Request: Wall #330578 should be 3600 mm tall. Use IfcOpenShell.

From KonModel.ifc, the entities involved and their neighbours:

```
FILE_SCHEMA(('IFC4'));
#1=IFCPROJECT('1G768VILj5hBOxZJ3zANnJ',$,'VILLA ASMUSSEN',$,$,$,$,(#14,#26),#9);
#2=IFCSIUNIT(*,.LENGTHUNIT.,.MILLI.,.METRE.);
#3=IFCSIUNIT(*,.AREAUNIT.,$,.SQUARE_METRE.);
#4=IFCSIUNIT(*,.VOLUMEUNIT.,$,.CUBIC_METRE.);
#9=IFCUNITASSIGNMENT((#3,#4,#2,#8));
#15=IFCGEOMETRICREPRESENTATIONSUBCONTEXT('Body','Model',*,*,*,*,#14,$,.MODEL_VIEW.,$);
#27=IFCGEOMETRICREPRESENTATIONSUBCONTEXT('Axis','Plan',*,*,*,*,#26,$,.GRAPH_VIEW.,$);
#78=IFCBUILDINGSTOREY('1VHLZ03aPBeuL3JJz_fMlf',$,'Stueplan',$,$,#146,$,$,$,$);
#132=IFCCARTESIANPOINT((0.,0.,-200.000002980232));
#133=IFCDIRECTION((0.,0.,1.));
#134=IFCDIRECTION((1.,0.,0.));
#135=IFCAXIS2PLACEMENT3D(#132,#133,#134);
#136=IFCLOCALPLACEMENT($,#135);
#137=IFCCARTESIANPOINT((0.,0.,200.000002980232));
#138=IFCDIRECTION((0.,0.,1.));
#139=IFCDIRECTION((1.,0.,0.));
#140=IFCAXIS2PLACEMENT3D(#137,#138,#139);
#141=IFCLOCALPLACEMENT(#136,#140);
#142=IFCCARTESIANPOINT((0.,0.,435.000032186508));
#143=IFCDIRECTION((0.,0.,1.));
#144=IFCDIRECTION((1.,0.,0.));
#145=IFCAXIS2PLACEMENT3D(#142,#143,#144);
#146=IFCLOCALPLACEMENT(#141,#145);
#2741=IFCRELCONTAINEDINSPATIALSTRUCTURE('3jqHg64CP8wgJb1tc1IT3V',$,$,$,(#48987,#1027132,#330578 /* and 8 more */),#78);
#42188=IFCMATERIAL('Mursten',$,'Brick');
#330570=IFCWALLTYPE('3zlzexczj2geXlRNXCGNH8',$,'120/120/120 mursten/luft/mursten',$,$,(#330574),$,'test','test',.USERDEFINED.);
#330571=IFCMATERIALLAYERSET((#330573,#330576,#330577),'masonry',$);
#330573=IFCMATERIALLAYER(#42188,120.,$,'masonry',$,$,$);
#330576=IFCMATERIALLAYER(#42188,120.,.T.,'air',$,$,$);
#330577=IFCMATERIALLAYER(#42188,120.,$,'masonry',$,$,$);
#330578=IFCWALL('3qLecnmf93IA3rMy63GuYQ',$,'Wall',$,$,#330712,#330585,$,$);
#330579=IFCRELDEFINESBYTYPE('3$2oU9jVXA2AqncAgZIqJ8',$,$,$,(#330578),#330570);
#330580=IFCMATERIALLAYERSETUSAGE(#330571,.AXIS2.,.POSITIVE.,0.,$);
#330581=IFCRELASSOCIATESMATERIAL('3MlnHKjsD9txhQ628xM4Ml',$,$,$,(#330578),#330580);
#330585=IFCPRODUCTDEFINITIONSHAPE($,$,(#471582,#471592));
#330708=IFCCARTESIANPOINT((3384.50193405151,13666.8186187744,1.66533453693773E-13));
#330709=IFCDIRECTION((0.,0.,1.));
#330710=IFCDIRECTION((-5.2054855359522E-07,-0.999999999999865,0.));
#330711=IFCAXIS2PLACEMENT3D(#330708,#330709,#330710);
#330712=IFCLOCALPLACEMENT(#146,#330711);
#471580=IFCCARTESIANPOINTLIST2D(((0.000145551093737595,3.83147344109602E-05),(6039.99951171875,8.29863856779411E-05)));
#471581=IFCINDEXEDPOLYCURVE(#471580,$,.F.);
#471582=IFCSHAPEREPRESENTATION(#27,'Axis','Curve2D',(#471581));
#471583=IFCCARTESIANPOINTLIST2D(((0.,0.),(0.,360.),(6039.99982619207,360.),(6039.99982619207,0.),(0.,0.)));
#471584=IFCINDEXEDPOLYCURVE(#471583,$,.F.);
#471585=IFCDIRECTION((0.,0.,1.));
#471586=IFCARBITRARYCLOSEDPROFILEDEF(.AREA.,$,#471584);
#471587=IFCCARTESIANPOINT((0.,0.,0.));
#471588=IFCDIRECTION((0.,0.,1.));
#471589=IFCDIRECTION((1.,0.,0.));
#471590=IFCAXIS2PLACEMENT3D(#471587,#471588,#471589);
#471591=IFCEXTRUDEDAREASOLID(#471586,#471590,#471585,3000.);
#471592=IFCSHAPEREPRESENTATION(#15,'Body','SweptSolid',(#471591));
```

```python
import ifcopenshell
import ifcopenshell.geom
import ifcopenshell.util.representation
import ifcopenshell.util.shape

model = ifcopenshell.open("KonModel.ifc")
settings = ifcopenshell.geom.settings()


def volume(element):
    """Net volume in cubic metres, openings subtracted."""
    shape = ifcopenshell.geom.create_shape(settings, element)
    return ifcopenshell.util.shape.get_volume(shape.geometry)


wall = model.by_guid("3qLecnmf93IA3rMy63GuYQ")
before = volume(wall)

body = ifcopenshell.util.representation.get_representation(wall, "Model", "Body")
solid = body.Items[0]
old_height = solid.Depth
solid.Depth = 3600.0
after = volume(wall)

print(f"height {old_height:g} -> {solid.Depth:g}, volume {before:.3f} -> {after:.3f} m3")

model.write("KonModel_rev.ifc")
```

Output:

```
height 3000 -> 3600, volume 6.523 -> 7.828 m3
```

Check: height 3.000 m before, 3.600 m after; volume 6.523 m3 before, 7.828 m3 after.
